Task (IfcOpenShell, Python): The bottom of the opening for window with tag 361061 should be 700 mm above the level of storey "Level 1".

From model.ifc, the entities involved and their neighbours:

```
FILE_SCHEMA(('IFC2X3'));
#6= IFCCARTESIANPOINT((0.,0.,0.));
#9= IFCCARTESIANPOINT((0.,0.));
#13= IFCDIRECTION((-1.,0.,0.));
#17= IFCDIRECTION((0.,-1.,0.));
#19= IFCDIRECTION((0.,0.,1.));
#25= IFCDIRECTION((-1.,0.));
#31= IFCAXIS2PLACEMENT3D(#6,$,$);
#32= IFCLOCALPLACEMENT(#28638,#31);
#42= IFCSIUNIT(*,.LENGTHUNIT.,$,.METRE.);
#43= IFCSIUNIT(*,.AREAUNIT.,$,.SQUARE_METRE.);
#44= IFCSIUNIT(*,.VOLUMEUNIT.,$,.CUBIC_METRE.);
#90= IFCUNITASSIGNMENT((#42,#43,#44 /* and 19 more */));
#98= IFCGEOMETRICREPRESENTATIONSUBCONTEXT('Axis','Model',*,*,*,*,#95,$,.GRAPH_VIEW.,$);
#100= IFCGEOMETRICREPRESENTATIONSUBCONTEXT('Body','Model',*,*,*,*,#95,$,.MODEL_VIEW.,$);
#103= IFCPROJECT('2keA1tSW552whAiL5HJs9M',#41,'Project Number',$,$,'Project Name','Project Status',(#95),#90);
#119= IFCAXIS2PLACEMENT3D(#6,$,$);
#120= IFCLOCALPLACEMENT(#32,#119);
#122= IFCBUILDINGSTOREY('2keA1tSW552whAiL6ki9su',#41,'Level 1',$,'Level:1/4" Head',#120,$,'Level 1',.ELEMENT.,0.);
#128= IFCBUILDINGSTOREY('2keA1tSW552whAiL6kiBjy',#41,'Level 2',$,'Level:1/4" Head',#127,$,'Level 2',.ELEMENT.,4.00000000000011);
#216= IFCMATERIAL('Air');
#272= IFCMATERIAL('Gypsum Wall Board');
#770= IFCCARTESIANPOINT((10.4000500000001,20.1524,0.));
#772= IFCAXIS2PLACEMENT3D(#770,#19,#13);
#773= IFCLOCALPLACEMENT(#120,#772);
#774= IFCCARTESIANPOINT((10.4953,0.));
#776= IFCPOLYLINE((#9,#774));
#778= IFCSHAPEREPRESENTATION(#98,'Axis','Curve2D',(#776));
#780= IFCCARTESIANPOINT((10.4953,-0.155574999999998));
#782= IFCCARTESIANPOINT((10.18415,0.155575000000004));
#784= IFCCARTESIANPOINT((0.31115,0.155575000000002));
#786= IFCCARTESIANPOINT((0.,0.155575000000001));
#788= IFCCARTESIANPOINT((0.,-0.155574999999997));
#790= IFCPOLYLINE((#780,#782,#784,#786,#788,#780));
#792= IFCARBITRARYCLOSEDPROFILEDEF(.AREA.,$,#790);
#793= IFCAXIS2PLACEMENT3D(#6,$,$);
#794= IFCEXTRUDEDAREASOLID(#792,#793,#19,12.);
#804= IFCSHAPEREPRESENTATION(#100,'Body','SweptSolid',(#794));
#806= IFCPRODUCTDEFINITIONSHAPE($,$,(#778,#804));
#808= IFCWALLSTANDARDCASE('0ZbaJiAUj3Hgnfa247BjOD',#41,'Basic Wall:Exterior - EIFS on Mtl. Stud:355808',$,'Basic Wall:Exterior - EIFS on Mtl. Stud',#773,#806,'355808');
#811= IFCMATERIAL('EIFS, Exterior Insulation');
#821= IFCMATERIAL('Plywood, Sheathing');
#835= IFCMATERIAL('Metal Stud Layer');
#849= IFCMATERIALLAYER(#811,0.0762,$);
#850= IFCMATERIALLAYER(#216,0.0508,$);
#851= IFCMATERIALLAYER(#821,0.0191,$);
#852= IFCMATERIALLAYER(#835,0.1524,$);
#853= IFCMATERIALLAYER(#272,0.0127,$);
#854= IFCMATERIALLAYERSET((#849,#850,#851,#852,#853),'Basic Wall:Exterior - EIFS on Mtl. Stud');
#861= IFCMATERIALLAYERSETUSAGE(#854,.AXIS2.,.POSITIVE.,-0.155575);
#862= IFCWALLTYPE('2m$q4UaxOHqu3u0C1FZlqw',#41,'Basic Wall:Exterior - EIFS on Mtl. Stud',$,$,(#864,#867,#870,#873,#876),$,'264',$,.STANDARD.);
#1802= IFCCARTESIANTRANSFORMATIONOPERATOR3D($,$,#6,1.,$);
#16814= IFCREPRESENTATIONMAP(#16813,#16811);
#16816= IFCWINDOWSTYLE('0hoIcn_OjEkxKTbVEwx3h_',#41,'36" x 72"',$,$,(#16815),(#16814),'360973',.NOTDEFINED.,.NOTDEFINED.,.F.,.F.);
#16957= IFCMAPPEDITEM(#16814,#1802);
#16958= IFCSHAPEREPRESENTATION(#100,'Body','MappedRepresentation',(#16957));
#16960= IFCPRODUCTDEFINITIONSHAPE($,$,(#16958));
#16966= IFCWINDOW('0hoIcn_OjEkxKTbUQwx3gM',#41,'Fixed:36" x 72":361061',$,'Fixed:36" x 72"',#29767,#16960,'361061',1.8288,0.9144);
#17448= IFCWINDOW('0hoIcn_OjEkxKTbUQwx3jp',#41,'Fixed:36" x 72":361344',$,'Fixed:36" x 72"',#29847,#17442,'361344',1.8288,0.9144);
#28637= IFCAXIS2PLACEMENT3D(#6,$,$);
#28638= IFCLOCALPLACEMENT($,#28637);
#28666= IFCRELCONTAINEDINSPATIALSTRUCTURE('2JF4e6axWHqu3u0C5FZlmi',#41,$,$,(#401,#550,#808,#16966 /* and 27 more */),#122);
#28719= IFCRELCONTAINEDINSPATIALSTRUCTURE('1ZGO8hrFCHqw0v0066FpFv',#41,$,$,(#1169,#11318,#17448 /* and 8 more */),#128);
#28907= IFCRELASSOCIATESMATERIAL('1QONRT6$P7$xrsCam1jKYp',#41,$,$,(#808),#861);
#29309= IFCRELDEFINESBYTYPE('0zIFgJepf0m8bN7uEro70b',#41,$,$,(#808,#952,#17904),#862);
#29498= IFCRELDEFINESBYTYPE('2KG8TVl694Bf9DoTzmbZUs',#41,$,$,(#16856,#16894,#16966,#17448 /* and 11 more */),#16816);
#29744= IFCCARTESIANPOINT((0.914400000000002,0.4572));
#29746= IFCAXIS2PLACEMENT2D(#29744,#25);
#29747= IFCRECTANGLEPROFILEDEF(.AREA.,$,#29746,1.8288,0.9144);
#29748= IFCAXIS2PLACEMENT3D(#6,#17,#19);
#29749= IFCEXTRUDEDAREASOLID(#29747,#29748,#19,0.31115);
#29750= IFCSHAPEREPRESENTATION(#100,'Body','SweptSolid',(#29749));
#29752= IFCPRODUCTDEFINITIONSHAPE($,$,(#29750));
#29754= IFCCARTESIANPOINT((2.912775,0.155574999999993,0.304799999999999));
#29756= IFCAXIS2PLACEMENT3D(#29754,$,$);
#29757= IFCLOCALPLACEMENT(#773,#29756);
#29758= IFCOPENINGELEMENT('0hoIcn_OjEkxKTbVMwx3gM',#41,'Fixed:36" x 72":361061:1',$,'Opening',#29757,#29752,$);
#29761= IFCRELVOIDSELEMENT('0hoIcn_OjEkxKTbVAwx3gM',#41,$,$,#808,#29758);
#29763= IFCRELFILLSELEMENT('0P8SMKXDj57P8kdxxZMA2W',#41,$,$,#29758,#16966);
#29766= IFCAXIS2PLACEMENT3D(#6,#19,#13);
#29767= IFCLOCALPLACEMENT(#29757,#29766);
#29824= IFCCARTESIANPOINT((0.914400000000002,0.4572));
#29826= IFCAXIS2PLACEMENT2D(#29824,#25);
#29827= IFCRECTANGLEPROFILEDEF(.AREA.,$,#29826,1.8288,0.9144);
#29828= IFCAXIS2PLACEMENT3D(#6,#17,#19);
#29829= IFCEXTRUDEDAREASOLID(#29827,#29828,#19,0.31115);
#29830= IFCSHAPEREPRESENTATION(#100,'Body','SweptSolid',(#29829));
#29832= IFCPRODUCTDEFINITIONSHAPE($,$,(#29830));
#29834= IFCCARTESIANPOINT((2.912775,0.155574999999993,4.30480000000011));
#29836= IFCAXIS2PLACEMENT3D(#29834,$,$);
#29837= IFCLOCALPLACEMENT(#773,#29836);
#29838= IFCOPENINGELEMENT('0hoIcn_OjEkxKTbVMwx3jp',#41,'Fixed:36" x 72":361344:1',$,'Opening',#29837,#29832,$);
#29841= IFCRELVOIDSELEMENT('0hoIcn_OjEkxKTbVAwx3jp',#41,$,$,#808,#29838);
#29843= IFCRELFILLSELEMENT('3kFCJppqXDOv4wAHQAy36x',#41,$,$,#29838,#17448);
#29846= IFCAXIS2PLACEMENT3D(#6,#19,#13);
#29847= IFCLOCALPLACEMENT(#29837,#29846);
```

```python
import numpy as np
import ifcopenshell
import ifcopenshell.api.geometry
import ifcopenshell.geom
import ifcopenshell.util.element
import ifcopenshell.util.placement
import ifcopenshell.util.shape
import ifcopenshell.util.unit

model = ifcopenshell.open("model.ifc")
unit_scale = ifcopenshell.util.unit.calculate_unit_scale(model)

window = model.by_guid("0hoIcn_OjEkxKTbUQwx3gM")
opening = window.FillsVoids[0].RelatingOpeningElement
storey = ifcopenshell.util.element.get_container(window, ifc_class="IfcBuildingStorey")
level = ifcopenshell.util.placement.get_local_placement(storey.ObjectPlacement)[2, 3]

# The opening's origin need not be at the sill, so measure its lowest point.
shape = ifcopenshell.geom.create_shape(ifcopenshell.geom.settings(), opening)
bottom = ifcopenshell.util.shape.get_shape_bottom_elevation(shape, shape.geometry) / unit_scale
dz = level + 0.7 / unit_scale - bottom

shift = np.array([0.0, 0.0, dz])
# The window is placed relative to its opening, so it follows when the opening moves.
matrix = ifcopenshell.util.placement.get_local_placement(opening.ObjectPlacement)
matrix[:3, 3] += shift
ifcopenshell.api.geometry.edit_object_placement(
    model, product=opening, matrix=matrix, is_si=False, should_transform_children=True
)

print(f"moved by {dz * unit_scale:+.3f} m")

model.write("model_edited.ifc")
```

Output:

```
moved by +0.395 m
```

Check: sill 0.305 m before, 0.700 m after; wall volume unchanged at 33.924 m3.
